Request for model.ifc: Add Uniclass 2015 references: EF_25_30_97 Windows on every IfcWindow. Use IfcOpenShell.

First a look at what the model holds.

```python
import ifcopenshell

model = ifcopenshell.open("model.ifc")
print(model.schema)
print("classifications:", [c.Name for c in model.by_type("IfcClassification")])
for ifc_class in ("IfcDoor", "IfcRoof", "IfcStair", "IfcWall", "IfcWindow"):
    print(ifc_class, len(model.by_type(ifc_class)))
```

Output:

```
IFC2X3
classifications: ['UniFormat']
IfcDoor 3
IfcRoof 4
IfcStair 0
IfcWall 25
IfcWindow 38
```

```python
import ifcopenshell
import ifcopenshell.api.classification

model = ifcopenshell.open("model.ifc")

# IFC2X3 requires Source and Edition and has no link from the project to the system.
system = model.create_entity("IfcClassification", Source="NBS", Edition="2015", Name="Uniclass 2015")

codes = {
    "IfcWindow": ("EF_25_30_97", "Windows"),
}
for ifc_class, (code, name) in codes.items():
    products = model.by_type(ifc_class)
    ifcopenshell.api.classification.add_reference(
        model, products=products, classification=system, identification=code, name=name
    )
    print(code, len(products))

model.write("model_edited.ifc")
```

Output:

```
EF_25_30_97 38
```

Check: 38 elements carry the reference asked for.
